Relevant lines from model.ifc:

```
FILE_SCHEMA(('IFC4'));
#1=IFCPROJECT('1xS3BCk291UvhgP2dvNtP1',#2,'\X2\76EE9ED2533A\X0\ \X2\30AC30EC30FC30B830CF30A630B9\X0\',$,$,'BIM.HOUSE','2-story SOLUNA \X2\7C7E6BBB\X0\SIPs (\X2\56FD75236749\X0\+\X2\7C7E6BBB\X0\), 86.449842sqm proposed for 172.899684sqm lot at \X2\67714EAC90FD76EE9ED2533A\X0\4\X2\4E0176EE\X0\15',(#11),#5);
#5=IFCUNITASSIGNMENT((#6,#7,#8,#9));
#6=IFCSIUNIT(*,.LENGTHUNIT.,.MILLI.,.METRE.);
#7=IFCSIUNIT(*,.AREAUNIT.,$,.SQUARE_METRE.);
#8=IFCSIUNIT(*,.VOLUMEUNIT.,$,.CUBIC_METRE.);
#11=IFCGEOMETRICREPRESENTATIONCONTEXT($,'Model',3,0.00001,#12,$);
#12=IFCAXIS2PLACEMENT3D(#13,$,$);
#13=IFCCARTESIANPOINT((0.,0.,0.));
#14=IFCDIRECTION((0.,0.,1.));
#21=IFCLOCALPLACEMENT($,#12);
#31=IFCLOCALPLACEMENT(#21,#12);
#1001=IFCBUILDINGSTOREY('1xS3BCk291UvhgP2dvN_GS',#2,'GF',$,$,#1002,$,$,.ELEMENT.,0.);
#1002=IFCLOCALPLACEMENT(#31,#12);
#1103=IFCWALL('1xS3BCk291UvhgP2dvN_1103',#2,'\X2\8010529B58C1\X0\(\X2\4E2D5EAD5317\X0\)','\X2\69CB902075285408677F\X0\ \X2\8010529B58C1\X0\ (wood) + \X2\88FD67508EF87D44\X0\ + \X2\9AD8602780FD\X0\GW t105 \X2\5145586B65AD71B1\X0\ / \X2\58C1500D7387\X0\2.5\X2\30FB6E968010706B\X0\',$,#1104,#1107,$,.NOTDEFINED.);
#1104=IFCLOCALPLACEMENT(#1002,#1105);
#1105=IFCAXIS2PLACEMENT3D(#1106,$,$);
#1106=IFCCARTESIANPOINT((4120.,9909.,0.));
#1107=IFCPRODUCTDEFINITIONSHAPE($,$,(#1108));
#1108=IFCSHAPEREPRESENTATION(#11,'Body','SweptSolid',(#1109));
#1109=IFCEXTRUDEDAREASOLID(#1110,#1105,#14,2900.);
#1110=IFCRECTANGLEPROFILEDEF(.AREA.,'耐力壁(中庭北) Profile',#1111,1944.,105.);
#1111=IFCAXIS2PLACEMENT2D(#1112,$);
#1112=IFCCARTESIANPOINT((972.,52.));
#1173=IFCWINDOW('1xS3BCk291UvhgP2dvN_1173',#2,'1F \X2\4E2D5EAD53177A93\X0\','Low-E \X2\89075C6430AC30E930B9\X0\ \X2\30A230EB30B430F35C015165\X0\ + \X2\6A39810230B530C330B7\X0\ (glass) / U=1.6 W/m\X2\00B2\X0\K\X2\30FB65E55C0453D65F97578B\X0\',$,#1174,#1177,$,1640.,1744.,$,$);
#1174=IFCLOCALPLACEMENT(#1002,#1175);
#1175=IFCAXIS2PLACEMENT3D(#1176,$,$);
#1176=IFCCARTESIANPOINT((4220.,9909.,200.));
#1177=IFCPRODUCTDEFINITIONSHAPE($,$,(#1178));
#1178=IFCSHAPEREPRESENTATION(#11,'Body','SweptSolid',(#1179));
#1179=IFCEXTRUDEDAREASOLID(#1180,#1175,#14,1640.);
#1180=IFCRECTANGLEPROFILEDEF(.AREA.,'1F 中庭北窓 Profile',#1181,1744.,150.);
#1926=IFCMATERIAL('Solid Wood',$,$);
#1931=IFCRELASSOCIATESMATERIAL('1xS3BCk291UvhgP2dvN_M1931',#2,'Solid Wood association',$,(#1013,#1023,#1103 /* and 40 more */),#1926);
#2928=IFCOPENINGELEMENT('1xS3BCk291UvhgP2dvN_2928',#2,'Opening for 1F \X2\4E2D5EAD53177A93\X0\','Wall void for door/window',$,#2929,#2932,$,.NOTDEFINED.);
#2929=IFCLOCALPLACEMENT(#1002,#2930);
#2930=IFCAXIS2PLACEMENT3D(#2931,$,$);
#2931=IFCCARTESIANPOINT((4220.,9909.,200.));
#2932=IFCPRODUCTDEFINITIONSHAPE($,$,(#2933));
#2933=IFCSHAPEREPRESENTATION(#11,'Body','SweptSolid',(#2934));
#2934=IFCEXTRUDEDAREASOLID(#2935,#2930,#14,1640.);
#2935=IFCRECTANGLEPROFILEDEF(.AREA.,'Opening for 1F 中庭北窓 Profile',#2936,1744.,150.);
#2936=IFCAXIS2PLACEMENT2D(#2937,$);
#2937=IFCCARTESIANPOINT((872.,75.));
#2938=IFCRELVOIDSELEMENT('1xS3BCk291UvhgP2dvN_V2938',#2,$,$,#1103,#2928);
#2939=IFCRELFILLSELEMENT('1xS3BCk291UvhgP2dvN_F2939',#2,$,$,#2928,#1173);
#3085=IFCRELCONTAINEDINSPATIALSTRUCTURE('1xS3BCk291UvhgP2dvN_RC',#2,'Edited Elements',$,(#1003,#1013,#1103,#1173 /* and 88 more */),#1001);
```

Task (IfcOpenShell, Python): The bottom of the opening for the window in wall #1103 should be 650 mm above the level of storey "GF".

```python
import numpy as np
import ifcopenshell
import ifcopenshell.api.geometry
import ifcopenshell.geom
import ifcopenshell.util.element
import ifcopenshell.util.placement
import ifcopenshell.util.shape
import ifcopenshell.util.unit

model = ifcopenshell.open("model.ifc")
unit_scale = ifcopenshell.util.unit.calculate_unit_scale(model)

window = model.by_guid("1xS3BCk291UvhgP2dvN_1173")
opening = window.FillsVoids[0].RelatingOpeningElement
storey = ifcopenshell.util.element.get_container(window, ifc_class="IfcBuildingStorey")
level = ifcopenshell.util.placement.get_local_placement(storey.ObjectPlacement)[2, 3]

# The opening's origin need not be at the sill, so measure its lowest point.
shape = ifcopenshell.geom.create_shape(ifcopenshell.geom.settings(), opening)
bottom = ifcopenshell.util.shape.get_shape_bottom_elevation(shape, shape.geometry) / unit_scale
dz = level + 650.0 - bottom

shift = np.array([0.0, 0.0, dz])
# The window is not placed relative to its opening, so move both.
for product in (opening, window):
    matrix = ifcopenshell.util.placement.get_local_placement(product.ObjectPlacement)
    matrix[:3, 3] += shift
    ifcopenshell.api.geometry.edit_object_placement(model, product=product, matrix=matrix, is_si=False)

print(f"moved by {dz * unit_scale:+.3f} m")

model.write("model_rev.ifc")
```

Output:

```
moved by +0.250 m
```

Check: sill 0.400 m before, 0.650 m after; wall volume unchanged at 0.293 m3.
